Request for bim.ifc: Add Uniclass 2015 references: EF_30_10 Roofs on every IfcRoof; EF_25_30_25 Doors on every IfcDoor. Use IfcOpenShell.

First a look at what the model holds.

```python
import ifcopenshell

model = ifcopenshell.open("bim.ifc")
print(model.schema)
print("classifications:", [c.Name for c in model.by_type("IfcClassification")])
for ifc_class in ("IfcDoor", "IfcRoof", "IfcStair", "IfcWall", "IfcWindow"):
    print(ifc_class, len(model.by_type(ifc_class)))
```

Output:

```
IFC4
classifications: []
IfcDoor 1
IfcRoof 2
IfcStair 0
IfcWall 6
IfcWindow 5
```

```python
import ifcopenshell
import ifcopenshell.api.classification

model = ifcopenshell.open("bim.ifc")

system = ifcopenshell.api.classification.add_classification(model, classification="Uniclass 2015")

codes = {
    "IfcRoof": ("EF_30_10", "Roofs"),
    "IfcDoor": ("EF_25_30_25", "Doors"),
}
for ifc_class, (code, name) in codes.items():
    products = model.by_type(ifc_class)
    ifcopenshell.api.classification.add_reference(
        model, products=products, classification=system, identification=code, name=name
    )
    print(code, len(products))

model.write("bim_v2.ifc")
```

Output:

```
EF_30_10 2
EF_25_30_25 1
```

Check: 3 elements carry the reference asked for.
